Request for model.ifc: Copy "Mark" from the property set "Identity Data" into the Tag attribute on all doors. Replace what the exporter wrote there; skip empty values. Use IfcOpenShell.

First a look at what the model holds.

```python
import ifcopenshell
import ifcopenshell.util.element

model = ifcopenshell.open("model.ifc")
print(model.schema)
doors = model.by_type("IfcDoor")
print(len(doors), "doors")
for e in doors[:8]:
    source = ifcopenshell.util.element.get_pset(e, "Identity Data", "Mark")
    target = e.Tag
    print(e.id(), repr(source), repr(target), sep=" | ")
```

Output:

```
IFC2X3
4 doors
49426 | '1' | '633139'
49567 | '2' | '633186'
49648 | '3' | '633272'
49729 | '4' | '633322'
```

```python
import ifcopenshell
import ifcopenshell.util.element

model = ifcopenshell.open("model.ifc")

count = 0
for e in model.by_type("IfcDoor"):
    value = ifcopenshell.util.element.get_pset(e, "Identity Data", "Mark")
    current = e.Tag
    if not value or not value.strip() or current == value:
        continue
    e.Tag = value
    count += 1

print(count, "doors updated")

model.write("model-out.ifc")
```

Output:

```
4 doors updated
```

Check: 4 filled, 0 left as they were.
